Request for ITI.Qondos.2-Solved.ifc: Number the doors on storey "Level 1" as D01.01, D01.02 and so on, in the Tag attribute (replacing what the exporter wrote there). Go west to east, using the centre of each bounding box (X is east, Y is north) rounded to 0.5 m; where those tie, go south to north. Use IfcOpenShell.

First a look at what the model holds.

```python
import ifcopenshell
import ifcopenshell.util.element
import ifcopenshell.util.placement

model = ifcopenshell.open("ITI.Qondos.2-Solved.ifc")
print(model.schema)
storey = next(s for s in model.by_type("IfcBuildingStorey") if s.Name == "Level 1")
doors = [e for e in ifcopenshell.util.element.get_decomposition(storey) if e.is_a("IfcDoor")]
for e in sorted(doors, key=lambda e: e.id()):
    origin = ifcopenshell.util.placement.get_local_placement(e.ObjectPlacement)[:3, 3]
    print(e.id(), e.Tag, e.Name, origin.round(2) + 0.0, sep=" | ")
```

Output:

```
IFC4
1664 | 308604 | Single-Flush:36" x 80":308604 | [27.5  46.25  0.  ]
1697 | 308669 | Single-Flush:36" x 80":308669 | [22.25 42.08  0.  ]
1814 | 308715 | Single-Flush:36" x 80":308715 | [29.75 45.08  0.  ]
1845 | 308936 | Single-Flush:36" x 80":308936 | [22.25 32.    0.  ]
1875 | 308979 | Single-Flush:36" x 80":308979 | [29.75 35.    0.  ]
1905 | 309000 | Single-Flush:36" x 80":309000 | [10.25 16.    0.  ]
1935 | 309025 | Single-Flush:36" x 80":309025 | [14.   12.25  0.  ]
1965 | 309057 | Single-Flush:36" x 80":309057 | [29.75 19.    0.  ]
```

```python
import ifcopenshell
import ifcopenshell.geom
import ifcopenshell.util.element
import ifcopenshell.util.shape

model = ifcopenshell.open("ITI.Qondos.2-Solved.ifc")
settings = ifcopenshell.geom.settings()
settings.set("use-world-coords", True)


def centre(element):
    shape = ifcopenshell.geom.create_shape(settings, element)
    return ifcopenshell.util.shape.get_bbox_centroid(shape.geometry)


storey = next(s for s in model.by_type("IfcBuildingStorey") if s.Name == "Level 1")
doors = [e for e in ifcopenshell.util.element.get_decomposition(storey) if e.is_a("IfcDoor")]

# Insertion points can sit at a corner or the storey origin, so sort by the geometry (in metres).
centres = {e: centre(e) for e in doors}
doors.sort(key=lambda e: (round(centres[e][0] / 0.5), centres[e][1]))

for i, e in enumerate(doors, start=1):
    number = f"D01.{i:02d}"
    e.Tag = number
    print(e.id(), number)

model.write("ITI.Qondos.2-Solved_updated.ifc")
```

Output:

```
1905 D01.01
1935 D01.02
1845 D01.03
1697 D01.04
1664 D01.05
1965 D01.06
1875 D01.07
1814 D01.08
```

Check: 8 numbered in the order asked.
